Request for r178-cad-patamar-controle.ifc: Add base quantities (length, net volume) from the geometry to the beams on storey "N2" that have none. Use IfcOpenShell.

First a look at what the model holds.

```python
import ifcopenshell
import ifcopenshell.util.element
import ifcopenshell.util.unit

model = ifcopenshell.open("r178-cad-patamar-controle.ifc")
print(model.schema)
for unit_type in ("LENGTHUNIT", "AREAUNIT", "VOLUMEUNIT"):
    print(unit_type, ifcopenshell.util.unit.calculate_unit_scale(model, unit_type))
storey = next(s for s in model.by_type("IfcBuildingStorey") if s.Name == "N2")
beams = [e for e in ifcopenshell.util.element.get_decomposition(storey) if e.is_a("IfcBeam")]
for e in sorted(beams, key=lambda e: e.id()):
    print(e.id(), e.is_a(), e.Name, list(ifcopenshell.util.element.get_psets(e, qtos_only=True)), sep=" | ")
```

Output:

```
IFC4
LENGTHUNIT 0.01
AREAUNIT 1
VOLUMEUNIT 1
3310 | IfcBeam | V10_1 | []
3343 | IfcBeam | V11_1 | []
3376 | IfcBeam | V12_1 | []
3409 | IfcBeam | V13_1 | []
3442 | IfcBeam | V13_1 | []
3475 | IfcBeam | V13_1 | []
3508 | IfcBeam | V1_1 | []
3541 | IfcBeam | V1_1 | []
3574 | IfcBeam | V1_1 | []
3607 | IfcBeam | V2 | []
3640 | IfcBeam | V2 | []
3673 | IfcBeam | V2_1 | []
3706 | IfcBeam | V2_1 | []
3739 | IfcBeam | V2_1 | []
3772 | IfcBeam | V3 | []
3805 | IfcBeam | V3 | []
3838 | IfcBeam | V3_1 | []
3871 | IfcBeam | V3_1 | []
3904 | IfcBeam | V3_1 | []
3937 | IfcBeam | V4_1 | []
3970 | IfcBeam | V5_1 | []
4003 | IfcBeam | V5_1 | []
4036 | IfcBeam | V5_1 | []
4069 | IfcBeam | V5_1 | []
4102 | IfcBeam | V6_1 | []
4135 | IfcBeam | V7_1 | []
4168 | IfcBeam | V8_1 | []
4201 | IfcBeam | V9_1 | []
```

```python
import ifcopenshell
import ifcopenshell.api.pset
import ifcopenshell.geom
import ifcopenshell.util.element
import ifcopenshell.util.shape
import ifcopenshell.util.unit

model = ifcopenshell.open("r178-cad-patamar-controle.ifc")
unit_scale = ifcopenshell.util.unit.calculate_unit_scale(model)
volume_scale = ifcopenshell.util.unit.calculate_unit_scale(model, "VOLUMEUNIT")
settings = ifcopenshell.geom.settings()

storey = next(s for s in model.by_type("IfcBuildingStorey") if s.Name == "N2")
beams = [e for e in ifcopenshell.util.element.get_decomposition(storey) if e.is_a("IfcBeam")]

for e in sorted(beams, key=lambda e: e.id()):
    if ifcopenshell.util.element.get_psets(e, qtos_only=True, should_inherit=False):
        continue
    # Geometry comes back in metres, in the element's own axes.
    shape = ifcopenshell.geom.create_shape(settings, e)
    values = {
        "Length": ifcopenshell.util.shape.get_max_xyz(shape.geometry) / unit_scale,
        "NetVolume": ifcopenshell.util.shape.get_volume(shape.geometry) / volume_scale,
    }
    qto = ifcopenshell.api.pset.add_qto(model, product=e, name="Qto_BeamBaseQuantities")
    ifcopenshell.api.pset.edit_qto(model, qto=qto, properties=values)
    print(e.id(), {k: round(v, 3) for k, v in values.items()})

model.write("r178-cad-patamar-controle_edited.ifc")
```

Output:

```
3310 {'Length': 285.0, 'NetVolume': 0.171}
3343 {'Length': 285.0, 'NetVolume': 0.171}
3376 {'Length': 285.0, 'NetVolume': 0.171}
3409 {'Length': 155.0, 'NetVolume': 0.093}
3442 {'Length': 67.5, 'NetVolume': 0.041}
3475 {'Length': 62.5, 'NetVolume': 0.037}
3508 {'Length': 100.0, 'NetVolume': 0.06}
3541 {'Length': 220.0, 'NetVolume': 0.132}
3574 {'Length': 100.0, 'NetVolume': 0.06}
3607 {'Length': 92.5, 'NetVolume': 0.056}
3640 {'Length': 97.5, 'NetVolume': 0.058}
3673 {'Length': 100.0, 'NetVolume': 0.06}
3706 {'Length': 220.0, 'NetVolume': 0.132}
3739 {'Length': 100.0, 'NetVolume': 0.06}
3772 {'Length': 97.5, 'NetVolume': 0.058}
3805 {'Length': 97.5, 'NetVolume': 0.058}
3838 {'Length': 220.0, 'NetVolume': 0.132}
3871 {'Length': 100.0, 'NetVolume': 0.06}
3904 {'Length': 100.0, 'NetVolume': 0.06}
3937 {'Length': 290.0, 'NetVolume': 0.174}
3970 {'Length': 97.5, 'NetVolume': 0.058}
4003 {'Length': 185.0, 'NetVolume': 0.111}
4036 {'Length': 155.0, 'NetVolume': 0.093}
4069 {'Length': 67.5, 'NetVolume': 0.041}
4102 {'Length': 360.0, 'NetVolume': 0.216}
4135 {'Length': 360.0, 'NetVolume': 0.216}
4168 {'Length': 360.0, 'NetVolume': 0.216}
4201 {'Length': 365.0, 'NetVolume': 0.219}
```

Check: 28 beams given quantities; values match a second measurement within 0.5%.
